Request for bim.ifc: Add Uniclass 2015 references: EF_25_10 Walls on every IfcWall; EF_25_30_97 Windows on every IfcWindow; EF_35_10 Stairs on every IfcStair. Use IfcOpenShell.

First a look at what the model holds.

```python
import ifcopenshell

model = ifcopenshell.open("bim.ifc")
print(model.schema)
print("classifications:", [c.Name for c in model.by_type("IfcClassification")])
for ifc_class in ("IfcDoor", "IfcRoof", "IfcStair", "IfcWall", "IfcWindow"):
    print(ifc_class, len(model.by_type(ifc_class)))
```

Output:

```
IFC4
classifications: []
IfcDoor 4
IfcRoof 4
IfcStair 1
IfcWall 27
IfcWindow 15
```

```python
import ifcopenshell
import ifcopenshell.api.classification

model = ifcopenshell.open("bim.ifc")

system = ifcopenshell.api.classification.add_classification(model, classification="Uniclass 2015")

codes = {
    "IfcWall": ("EF_25_10", "Walls"),
    "IfcWindow": ("EF_25_30_97", "Windows"),
    "IfcStair": ("EF_35_10", "Stairs"),
}
for ifc_class, (code, name) in codes.items():
    products = model.by_type(ifc_class)
    ifcopenshell.api.classification.add_reference(
        model, products=products, classification=system, identification=code, name=name
    )
    print(code, len(products))

model.write("bim-out.ifc")
```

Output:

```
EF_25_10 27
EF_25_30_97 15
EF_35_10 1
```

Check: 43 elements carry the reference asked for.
